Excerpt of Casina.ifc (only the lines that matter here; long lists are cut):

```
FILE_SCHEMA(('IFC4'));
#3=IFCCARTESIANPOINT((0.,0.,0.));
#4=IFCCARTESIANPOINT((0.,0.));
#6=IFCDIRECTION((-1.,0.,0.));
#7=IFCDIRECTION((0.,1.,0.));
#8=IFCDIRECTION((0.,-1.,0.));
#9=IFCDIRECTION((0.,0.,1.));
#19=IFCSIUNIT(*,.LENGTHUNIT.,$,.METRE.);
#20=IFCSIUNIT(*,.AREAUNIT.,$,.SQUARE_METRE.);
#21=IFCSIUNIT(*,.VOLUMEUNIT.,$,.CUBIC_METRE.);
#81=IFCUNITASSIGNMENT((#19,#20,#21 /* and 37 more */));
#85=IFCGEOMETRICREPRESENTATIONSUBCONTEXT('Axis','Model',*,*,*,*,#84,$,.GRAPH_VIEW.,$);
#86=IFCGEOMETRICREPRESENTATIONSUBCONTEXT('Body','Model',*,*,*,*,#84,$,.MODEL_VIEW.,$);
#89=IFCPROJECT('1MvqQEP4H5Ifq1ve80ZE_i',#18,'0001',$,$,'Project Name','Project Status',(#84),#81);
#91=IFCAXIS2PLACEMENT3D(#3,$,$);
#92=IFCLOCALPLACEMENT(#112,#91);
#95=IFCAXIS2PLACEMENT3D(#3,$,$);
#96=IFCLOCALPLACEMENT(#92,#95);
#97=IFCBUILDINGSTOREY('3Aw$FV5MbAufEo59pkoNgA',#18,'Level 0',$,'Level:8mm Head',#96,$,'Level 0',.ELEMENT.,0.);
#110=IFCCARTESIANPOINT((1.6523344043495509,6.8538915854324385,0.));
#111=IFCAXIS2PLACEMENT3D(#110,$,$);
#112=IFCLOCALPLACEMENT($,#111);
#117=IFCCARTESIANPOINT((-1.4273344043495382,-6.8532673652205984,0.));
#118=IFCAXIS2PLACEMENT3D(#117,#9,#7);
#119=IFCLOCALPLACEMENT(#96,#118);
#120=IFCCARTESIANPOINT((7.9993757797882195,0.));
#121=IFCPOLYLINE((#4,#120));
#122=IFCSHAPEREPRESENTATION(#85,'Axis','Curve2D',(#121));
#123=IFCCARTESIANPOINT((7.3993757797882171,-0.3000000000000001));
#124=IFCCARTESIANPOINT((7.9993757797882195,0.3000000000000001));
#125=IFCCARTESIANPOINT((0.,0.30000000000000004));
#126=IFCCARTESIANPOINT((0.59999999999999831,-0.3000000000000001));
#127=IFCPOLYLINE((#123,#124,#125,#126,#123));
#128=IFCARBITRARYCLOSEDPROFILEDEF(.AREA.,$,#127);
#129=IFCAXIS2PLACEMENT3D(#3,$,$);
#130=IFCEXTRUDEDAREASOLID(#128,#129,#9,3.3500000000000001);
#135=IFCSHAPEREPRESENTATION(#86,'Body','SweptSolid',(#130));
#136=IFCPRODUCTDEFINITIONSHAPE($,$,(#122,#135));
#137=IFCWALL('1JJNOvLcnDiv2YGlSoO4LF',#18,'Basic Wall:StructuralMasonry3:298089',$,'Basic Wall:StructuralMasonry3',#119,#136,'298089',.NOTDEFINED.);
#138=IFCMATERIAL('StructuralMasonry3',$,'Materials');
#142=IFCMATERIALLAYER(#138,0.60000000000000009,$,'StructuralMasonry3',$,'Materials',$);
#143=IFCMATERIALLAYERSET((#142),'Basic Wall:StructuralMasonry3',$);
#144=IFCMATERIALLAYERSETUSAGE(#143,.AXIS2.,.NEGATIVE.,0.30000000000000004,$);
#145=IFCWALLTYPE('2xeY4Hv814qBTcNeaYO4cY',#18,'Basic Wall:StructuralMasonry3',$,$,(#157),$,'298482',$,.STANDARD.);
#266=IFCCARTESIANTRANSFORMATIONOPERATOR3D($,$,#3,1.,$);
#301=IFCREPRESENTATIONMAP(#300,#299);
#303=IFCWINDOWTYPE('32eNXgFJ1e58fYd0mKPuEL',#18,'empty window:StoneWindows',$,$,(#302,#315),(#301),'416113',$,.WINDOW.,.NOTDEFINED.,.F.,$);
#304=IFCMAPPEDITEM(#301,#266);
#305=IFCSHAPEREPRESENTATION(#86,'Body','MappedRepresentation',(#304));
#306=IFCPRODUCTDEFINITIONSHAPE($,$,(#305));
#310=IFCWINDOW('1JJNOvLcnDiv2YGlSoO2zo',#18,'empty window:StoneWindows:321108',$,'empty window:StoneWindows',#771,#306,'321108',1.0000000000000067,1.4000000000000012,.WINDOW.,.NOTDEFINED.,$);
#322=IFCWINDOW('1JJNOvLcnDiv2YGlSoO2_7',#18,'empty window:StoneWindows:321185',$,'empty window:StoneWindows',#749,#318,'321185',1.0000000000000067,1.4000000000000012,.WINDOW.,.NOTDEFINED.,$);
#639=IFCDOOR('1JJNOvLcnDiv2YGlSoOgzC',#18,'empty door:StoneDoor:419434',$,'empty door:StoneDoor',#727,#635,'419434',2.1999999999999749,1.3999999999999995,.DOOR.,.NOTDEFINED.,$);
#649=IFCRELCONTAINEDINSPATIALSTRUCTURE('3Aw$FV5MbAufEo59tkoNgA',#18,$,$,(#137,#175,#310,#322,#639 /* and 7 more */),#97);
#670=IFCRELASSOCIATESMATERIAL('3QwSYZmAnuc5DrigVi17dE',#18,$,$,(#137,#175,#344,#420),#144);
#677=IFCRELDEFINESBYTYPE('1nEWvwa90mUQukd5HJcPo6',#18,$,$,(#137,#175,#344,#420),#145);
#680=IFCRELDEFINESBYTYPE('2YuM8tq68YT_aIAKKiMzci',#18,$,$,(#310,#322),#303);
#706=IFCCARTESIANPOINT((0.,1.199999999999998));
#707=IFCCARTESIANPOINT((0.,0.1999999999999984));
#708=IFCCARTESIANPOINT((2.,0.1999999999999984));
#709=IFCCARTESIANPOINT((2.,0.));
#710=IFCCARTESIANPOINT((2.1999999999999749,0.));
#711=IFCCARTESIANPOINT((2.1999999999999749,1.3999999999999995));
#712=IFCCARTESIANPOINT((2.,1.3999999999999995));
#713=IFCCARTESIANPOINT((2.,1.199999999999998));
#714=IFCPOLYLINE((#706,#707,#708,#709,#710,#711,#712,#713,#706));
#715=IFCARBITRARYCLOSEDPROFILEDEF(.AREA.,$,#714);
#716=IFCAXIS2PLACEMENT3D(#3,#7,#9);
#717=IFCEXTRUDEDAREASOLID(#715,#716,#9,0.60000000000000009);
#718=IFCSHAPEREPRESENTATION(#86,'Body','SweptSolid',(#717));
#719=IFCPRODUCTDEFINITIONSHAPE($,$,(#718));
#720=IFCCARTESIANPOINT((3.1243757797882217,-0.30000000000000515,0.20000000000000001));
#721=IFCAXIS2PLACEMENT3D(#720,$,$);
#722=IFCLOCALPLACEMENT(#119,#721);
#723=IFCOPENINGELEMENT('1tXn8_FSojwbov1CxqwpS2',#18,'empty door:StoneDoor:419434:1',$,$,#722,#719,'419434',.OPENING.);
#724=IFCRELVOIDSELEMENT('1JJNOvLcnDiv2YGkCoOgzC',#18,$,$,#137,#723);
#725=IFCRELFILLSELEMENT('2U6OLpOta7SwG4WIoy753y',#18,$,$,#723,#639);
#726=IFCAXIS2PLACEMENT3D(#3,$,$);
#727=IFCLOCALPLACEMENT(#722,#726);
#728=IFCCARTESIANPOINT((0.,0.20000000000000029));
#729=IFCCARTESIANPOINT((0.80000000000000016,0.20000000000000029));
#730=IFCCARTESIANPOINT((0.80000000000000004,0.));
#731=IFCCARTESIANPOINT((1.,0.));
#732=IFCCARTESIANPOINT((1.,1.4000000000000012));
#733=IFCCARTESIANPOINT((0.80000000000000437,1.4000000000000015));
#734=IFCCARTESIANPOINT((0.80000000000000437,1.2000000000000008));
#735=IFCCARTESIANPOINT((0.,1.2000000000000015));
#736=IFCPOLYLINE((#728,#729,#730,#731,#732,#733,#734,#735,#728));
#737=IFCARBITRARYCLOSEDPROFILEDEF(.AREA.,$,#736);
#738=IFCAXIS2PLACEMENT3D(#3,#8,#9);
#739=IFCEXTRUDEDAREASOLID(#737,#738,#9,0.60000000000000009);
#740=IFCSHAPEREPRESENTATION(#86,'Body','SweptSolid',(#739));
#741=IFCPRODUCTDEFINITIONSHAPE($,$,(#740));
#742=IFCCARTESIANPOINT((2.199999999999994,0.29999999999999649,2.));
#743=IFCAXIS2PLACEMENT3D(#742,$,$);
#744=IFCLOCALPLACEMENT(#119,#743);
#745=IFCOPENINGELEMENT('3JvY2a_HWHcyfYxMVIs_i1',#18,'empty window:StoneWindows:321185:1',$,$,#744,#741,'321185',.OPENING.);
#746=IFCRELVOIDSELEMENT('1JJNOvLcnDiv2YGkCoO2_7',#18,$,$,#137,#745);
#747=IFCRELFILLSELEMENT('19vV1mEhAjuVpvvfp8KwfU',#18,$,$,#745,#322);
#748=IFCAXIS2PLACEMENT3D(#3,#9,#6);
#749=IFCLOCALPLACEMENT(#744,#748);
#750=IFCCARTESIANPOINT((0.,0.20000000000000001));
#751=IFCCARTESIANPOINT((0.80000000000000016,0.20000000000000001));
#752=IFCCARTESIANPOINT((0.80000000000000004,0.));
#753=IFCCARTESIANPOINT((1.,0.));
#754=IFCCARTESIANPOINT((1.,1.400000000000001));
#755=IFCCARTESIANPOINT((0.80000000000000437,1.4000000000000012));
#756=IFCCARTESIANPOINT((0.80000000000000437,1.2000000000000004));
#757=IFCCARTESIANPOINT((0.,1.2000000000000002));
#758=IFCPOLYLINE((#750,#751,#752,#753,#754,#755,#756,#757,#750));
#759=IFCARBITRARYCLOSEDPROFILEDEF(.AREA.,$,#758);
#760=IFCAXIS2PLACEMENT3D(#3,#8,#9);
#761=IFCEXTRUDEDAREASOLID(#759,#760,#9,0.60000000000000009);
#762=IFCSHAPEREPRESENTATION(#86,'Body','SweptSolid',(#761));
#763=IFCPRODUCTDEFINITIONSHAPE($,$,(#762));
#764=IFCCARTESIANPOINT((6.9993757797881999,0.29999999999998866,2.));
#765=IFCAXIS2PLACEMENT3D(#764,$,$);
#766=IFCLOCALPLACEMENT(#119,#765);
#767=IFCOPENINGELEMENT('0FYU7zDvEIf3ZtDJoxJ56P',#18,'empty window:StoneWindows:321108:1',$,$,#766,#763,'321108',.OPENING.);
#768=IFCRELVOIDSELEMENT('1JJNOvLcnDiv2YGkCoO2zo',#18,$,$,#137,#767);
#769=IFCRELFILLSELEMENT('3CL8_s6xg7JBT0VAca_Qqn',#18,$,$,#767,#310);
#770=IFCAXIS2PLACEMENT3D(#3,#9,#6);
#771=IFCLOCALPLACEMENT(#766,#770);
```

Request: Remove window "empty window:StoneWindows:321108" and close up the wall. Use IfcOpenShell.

```python
import ifcopenshell
import ifcopenshell.api.feature
import ifcopenshell.api.root
import ifcopenshell.geom
import ifcopenshell.util.shape

model = ifcopenshell.open("Casina.ifc")
settings = ifcopenshell.geom.settings()


def volume(element):
    """Net volume in cubic metres, openings subtracted."""
    shape = ifcopenshell.geom.create_shape(settings, element)
    return ifcopenshell.util.shape.get_volume(shape.geometry)


window = model.by_id(310)
opening = window.FillsVoids[0].RelatingOpeningElement
wall = opening.VoidsElements[0].RelatingBuildingElement
before = volume(wall)

ifcopenshell.api.root.remove_product(model, product=window)
ifcopenshell.api.feature.remove_feature(model, feature=opening)

after = volume(wall)

print(f"wall volume {before:.3f} -> {after:.3f} m3")

model.write("Casina_updated.ifc")
```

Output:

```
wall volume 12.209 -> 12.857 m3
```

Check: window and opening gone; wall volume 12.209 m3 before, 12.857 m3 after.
